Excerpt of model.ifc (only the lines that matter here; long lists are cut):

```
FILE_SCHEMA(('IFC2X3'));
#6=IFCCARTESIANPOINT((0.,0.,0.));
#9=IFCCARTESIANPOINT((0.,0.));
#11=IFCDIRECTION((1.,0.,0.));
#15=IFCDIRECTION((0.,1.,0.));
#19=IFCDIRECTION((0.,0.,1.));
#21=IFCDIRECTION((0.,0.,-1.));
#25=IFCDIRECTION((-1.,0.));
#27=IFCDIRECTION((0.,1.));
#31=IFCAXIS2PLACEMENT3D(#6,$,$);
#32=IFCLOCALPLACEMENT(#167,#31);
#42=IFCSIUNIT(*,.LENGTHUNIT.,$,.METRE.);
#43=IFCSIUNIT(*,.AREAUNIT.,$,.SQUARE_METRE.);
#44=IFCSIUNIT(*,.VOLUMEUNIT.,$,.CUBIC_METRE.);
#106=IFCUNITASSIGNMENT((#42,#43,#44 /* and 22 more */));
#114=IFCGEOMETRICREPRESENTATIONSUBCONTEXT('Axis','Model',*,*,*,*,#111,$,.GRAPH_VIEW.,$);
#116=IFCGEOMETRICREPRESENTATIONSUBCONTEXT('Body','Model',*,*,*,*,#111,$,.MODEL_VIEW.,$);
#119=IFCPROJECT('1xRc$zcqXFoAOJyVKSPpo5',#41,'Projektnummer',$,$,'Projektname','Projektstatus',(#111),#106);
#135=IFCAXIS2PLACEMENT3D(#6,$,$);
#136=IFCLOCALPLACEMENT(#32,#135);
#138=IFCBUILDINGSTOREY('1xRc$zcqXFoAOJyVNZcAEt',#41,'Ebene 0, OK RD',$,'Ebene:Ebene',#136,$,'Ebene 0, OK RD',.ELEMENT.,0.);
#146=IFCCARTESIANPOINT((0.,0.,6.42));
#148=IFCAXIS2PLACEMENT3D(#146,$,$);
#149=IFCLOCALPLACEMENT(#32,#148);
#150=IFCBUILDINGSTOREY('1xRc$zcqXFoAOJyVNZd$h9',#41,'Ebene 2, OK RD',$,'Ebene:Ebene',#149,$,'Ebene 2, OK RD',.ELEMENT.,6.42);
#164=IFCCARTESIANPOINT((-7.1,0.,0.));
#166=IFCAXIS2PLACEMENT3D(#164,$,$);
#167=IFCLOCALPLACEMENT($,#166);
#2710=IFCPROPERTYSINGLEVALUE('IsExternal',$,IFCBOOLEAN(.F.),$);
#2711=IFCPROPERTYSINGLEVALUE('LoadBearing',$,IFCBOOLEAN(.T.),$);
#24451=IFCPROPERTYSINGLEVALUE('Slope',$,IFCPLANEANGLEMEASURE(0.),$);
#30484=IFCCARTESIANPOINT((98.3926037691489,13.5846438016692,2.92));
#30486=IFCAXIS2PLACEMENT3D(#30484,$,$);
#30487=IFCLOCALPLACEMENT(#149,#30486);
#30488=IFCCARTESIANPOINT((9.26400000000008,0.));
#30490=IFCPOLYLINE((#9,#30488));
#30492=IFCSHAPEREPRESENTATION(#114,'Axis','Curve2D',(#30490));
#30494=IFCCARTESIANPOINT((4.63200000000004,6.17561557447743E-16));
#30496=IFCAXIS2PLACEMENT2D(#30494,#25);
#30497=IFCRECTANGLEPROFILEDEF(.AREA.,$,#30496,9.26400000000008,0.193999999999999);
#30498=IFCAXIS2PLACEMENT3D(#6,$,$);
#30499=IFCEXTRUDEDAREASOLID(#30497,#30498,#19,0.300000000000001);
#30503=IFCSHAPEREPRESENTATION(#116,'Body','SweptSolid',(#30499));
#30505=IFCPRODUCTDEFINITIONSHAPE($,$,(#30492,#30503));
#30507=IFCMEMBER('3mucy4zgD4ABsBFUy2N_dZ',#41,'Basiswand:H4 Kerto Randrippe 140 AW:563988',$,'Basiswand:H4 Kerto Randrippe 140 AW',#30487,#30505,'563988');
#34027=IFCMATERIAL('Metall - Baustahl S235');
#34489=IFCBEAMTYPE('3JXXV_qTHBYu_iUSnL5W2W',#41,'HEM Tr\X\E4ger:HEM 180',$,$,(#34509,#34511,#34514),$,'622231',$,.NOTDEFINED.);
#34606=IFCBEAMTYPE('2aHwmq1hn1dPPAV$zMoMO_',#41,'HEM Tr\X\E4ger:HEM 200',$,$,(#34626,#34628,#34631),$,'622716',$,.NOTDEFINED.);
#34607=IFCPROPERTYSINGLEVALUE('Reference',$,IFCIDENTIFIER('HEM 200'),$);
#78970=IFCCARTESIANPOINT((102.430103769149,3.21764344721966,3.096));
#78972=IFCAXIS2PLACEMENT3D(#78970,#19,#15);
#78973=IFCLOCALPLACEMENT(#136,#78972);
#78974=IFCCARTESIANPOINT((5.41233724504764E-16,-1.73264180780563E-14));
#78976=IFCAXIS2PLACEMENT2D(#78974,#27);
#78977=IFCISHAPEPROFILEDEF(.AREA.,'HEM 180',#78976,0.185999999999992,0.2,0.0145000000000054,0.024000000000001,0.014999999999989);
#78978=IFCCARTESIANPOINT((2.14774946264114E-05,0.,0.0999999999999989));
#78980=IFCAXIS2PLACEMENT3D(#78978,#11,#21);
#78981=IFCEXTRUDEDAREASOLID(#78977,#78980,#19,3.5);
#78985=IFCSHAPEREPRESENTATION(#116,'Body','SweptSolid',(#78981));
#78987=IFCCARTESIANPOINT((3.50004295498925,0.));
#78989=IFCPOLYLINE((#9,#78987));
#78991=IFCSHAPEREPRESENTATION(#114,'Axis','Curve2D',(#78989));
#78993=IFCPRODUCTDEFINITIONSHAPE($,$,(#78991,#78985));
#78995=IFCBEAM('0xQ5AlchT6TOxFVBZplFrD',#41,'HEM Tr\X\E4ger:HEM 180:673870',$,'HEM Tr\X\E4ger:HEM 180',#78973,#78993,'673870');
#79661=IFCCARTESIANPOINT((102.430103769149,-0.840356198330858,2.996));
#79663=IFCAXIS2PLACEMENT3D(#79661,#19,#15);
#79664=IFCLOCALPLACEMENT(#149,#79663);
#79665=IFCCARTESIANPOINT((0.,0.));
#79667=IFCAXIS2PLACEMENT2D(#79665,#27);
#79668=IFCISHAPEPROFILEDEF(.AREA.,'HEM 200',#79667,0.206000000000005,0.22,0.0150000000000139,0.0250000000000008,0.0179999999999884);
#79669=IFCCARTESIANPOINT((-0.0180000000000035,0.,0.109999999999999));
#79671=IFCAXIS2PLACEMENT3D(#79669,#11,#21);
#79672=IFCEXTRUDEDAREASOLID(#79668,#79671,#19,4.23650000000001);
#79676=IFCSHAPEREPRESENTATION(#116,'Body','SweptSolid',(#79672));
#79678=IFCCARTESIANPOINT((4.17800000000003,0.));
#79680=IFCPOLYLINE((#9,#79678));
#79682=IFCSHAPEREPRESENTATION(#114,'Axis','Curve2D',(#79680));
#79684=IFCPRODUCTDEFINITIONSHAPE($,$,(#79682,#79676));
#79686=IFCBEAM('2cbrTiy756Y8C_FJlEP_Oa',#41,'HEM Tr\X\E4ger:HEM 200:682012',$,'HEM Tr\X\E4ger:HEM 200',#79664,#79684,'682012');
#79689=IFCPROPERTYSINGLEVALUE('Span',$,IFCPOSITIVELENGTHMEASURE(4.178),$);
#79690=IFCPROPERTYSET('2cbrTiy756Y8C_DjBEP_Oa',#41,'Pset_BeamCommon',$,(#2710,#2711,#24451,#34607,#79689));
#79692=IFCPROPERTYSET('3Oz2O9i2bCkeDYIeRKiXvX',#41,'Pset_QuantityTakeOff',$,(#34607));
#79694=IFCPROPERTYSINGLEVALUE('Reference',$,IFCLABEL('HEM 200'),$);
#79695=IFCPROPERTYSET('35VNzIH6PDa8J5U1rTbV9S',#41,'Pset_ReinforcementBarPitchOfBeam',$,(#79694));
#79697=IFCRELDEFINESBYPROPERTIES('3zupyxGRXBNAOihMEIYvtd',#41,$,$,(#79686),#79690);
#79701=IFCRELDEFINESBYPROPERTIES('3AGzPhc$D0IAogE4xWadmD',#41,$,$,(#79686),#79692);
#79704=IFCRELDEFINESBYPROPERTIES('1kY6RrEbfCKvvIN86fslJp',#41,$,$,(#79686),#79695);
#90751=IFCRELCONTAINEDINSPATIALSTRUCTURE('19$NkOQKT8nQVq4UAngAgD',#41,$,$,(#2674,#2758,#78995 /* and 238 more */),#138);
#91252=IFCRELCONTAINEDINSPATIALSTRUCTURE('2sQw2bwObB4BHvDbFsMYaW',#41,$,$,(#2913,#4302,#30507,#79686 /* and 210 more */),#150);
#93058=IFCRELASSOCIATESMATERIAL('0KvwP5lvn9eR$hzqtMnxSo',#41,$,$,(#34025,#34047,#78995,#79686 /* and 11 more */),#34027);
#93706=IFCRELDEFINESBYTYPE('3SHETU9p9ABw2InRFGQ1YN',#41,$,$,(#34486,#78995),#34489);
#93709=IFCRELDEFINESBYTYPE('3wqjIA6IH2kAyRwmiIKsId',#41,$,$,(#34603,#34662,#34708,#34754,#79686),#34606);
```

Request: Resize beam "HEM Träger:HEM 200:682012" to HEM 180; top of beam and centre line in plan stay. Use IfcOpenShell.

```python
import ifcopenshell
import ifcopenshell.api.pset
import ifcopenshell.api.type
import ifcopenshell.util.element
import ifcopenshell.util.representation

model = ifcopenshell.open("model.ifc")

member = model.by_guid("2cbrTiy756Y8C_FJlEP_Oa")
source = next(p for p in model.by_type("IfcIShapeProfileDef") if p.ProfileName == "HEM 180")

body = ifcopenshell.util.representation.get_representation(member, "Model", "Body")
solid = body.Items[0]
old_profile = solid.SweptArea

# Copy the section's sizes but keep this member's own profile position.
profile = ifcopenshell.util.element.copy(model, source)
# Profiles are centred, so shift by half the change in depth to hold the top.
shift = (old_profile.OverallDepth - profile.OverallDepth) / 2
x, y = old_profile.Position.Location.Coordinates
up = (-1.0, 0.0)  # upwards, in the solid's own plane
location = model.createIfcCartesianPoint((x + up[0] * shift, y + up[1] * shift))
profile.Position = model.createIfcAxis2Placement2D(location, old_profile.Position.RefDirection)
solid.SweptArea = profile
if not model.get_total_inverses(old_profile):
    ifcopenshell.util.element.remove_deep2(model, old_profile)

new_type = model.by_id(34489)
ifcopenshell.api.type.assign_type(
    model, related_objects=[member], relating_type=new_type, should_map_representations=False
)
member.Name = member.Name.replace("HEM 200", "HEM 180")
member.ObjectType = "HEM Träger:HEM 180"
pset = model.by_id(ifcopenshell.util.element.get_pset(member, "Pset_BeamCommon", should_inherit=False)["id"])
ifcopenshell.api.pset.edit_pset(model, pset=pset, properties={"Reference": "HEM 180"})
pset = model.by_id(ifcopenshell.util.element.get_pset(member, "Pset_QuantityTakeOff", should_inherit=False)["id"])
ifcopenshell.api.pset.edit_pset(model, pset=pset, properties={"Reference": "HEM 180"})
pset = model.by_id(ifcopenshell.util.element.get_pset(member, "Pset_ReinforcementBarPitchOfBeam", should_inherit=False)["id"])
ifcopenshell.api.pset.edit_pset(model, pset=pset, properties={"Reference": "HEM 180"})

print(solid.SweptArea)

model.write("model_rev.ifc")
```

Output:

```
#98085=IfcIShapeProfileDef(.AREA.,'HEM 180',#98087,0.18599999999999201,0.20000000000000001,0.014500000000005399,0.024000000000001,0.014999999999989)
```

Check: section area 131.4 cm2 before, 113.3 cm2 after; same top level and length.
